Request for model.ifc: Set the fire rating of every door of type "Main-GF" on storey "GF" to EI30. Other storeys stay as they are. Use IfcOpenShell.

First a look at what the model holds.

```python
import ifcopenshell
import ifcopenshell.util.element

model = ifcopenshell.open("model.ifc")
print(model.schema)
storey = next(s for s in model.by_type("IfcBuildingStorey") if s.Name == "GF")
doors = [e for e in ifcopenshell.util.element.get_decomposition(storey) if e.is_a("IfcDoor")]
seen = {}
for e in doors:
    element_type = ifcopenshell.util.element.get_type(e)
    key = (element_type.Name if element_type != e and element_type else None, ifcopenshell.util.element.get_pset(e, "Pset_DoorCommon", "FireRating"))
    seen[key] = seen.get(key, 0) + 1
for (name, value), count in sorted(seen.items(), key=str):
    print(count, "x", name, "|", value)
```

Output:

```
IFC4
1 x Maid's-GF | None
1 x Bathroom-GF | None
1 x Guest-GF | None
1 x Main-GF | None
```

```python
import ifcopenshell
import ifcopenshell.api.pset
import ifcopenshell.util.element

model = ifcopenshell.open("model.ifc")

storey = next(s for s in model.by_type("IfcBuildingStorey") if s.Name == "GF")
doors = [e for e in ifcopenshell.util.element.get_decomposition(storey) if e.is_a("IfcDoor")]

count = 0
for e in doors:
    element_type = ifcopenshell.util.element.get_type(e)
    if element_type in (None, e) or element_type.Name != "Main-GF":
        continue
    # add_pset returns the element's existing set when there is one.
    pset = ifcopenshell.api.pset.add_pset(model, product=e, name="Pset_DoorCommon")
    ifcopenshell.api.pset.edit_pset(model, pset=pset, properties={"FireRating": "EI30"})
    count += 1

print(count, "doors updated")

model.write("model-out.ifc")
```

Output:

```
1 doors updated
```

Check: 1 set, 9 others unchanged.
